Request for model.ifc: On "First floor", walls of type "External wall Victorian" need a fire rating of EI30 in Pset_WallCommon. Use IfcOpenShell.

First a look at what the model holds.

```python
import ifcopenshell
import ifcopenshell.util.element

model = ifcopenshell.open("model.ifc")
print(model.schema)
storey = next(s for s in model.by_type("IfcBuildingStorey") if s.Name == "First floor")
walls = [e for e in ifcopenshell.util.element.get_decomposition(storey) if e.is_a("IfcWall")]
seen = {}
for e in walls:
    element_type = ifcopenshell.util.element.get_type(e)
    key = (element_type.Name if element_type != e and element_type else None, ifcopenshell.util.element.get_pset(e, "Pset_WallCommon", "FireRating"))
    seen[key] = seen.get(key, 0) + 1
for (name, value), count in sorted(seen.items(), key=str):
    print(count, "x", name, "|", value)
```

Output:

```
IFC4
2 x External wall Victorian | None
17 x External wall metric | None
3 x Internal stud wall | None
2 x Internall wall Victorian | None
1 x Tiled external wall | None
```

```python
import ifcopenshell
import ifcopenshell.api.pset
import ifcopenshell.util.element

model = ifcopenshell.open("model.ifc")

storey = next(s for s in model.by_type("IfcBuildingStorey") if s.Name == "First floor")
walls = [e for e in ifcopenshell.util.element.get_decomposition(storey) if e.is_a("IfcWall")]

count = 0
for e in walls:
    element_type = ifcopenshell.util.element.get_type(e)
    if element_type in (None, e) or element_type.Name != "External wall Victorian":
        continue
    # add_pset returns the element's existing set when there is one.
    pset = ifcopenshell.api.pset.add_pset(model, product=e, name="Pset_WallCommon")
    ifcopenshell.api.pset.edit_pset(model, pset=pset, properties={"FireRating": "EI30"})
    count += 1

print(count, "walls updated")

model.write("model-out.ifc")
```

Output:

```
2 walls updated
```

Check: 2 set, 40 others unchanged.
